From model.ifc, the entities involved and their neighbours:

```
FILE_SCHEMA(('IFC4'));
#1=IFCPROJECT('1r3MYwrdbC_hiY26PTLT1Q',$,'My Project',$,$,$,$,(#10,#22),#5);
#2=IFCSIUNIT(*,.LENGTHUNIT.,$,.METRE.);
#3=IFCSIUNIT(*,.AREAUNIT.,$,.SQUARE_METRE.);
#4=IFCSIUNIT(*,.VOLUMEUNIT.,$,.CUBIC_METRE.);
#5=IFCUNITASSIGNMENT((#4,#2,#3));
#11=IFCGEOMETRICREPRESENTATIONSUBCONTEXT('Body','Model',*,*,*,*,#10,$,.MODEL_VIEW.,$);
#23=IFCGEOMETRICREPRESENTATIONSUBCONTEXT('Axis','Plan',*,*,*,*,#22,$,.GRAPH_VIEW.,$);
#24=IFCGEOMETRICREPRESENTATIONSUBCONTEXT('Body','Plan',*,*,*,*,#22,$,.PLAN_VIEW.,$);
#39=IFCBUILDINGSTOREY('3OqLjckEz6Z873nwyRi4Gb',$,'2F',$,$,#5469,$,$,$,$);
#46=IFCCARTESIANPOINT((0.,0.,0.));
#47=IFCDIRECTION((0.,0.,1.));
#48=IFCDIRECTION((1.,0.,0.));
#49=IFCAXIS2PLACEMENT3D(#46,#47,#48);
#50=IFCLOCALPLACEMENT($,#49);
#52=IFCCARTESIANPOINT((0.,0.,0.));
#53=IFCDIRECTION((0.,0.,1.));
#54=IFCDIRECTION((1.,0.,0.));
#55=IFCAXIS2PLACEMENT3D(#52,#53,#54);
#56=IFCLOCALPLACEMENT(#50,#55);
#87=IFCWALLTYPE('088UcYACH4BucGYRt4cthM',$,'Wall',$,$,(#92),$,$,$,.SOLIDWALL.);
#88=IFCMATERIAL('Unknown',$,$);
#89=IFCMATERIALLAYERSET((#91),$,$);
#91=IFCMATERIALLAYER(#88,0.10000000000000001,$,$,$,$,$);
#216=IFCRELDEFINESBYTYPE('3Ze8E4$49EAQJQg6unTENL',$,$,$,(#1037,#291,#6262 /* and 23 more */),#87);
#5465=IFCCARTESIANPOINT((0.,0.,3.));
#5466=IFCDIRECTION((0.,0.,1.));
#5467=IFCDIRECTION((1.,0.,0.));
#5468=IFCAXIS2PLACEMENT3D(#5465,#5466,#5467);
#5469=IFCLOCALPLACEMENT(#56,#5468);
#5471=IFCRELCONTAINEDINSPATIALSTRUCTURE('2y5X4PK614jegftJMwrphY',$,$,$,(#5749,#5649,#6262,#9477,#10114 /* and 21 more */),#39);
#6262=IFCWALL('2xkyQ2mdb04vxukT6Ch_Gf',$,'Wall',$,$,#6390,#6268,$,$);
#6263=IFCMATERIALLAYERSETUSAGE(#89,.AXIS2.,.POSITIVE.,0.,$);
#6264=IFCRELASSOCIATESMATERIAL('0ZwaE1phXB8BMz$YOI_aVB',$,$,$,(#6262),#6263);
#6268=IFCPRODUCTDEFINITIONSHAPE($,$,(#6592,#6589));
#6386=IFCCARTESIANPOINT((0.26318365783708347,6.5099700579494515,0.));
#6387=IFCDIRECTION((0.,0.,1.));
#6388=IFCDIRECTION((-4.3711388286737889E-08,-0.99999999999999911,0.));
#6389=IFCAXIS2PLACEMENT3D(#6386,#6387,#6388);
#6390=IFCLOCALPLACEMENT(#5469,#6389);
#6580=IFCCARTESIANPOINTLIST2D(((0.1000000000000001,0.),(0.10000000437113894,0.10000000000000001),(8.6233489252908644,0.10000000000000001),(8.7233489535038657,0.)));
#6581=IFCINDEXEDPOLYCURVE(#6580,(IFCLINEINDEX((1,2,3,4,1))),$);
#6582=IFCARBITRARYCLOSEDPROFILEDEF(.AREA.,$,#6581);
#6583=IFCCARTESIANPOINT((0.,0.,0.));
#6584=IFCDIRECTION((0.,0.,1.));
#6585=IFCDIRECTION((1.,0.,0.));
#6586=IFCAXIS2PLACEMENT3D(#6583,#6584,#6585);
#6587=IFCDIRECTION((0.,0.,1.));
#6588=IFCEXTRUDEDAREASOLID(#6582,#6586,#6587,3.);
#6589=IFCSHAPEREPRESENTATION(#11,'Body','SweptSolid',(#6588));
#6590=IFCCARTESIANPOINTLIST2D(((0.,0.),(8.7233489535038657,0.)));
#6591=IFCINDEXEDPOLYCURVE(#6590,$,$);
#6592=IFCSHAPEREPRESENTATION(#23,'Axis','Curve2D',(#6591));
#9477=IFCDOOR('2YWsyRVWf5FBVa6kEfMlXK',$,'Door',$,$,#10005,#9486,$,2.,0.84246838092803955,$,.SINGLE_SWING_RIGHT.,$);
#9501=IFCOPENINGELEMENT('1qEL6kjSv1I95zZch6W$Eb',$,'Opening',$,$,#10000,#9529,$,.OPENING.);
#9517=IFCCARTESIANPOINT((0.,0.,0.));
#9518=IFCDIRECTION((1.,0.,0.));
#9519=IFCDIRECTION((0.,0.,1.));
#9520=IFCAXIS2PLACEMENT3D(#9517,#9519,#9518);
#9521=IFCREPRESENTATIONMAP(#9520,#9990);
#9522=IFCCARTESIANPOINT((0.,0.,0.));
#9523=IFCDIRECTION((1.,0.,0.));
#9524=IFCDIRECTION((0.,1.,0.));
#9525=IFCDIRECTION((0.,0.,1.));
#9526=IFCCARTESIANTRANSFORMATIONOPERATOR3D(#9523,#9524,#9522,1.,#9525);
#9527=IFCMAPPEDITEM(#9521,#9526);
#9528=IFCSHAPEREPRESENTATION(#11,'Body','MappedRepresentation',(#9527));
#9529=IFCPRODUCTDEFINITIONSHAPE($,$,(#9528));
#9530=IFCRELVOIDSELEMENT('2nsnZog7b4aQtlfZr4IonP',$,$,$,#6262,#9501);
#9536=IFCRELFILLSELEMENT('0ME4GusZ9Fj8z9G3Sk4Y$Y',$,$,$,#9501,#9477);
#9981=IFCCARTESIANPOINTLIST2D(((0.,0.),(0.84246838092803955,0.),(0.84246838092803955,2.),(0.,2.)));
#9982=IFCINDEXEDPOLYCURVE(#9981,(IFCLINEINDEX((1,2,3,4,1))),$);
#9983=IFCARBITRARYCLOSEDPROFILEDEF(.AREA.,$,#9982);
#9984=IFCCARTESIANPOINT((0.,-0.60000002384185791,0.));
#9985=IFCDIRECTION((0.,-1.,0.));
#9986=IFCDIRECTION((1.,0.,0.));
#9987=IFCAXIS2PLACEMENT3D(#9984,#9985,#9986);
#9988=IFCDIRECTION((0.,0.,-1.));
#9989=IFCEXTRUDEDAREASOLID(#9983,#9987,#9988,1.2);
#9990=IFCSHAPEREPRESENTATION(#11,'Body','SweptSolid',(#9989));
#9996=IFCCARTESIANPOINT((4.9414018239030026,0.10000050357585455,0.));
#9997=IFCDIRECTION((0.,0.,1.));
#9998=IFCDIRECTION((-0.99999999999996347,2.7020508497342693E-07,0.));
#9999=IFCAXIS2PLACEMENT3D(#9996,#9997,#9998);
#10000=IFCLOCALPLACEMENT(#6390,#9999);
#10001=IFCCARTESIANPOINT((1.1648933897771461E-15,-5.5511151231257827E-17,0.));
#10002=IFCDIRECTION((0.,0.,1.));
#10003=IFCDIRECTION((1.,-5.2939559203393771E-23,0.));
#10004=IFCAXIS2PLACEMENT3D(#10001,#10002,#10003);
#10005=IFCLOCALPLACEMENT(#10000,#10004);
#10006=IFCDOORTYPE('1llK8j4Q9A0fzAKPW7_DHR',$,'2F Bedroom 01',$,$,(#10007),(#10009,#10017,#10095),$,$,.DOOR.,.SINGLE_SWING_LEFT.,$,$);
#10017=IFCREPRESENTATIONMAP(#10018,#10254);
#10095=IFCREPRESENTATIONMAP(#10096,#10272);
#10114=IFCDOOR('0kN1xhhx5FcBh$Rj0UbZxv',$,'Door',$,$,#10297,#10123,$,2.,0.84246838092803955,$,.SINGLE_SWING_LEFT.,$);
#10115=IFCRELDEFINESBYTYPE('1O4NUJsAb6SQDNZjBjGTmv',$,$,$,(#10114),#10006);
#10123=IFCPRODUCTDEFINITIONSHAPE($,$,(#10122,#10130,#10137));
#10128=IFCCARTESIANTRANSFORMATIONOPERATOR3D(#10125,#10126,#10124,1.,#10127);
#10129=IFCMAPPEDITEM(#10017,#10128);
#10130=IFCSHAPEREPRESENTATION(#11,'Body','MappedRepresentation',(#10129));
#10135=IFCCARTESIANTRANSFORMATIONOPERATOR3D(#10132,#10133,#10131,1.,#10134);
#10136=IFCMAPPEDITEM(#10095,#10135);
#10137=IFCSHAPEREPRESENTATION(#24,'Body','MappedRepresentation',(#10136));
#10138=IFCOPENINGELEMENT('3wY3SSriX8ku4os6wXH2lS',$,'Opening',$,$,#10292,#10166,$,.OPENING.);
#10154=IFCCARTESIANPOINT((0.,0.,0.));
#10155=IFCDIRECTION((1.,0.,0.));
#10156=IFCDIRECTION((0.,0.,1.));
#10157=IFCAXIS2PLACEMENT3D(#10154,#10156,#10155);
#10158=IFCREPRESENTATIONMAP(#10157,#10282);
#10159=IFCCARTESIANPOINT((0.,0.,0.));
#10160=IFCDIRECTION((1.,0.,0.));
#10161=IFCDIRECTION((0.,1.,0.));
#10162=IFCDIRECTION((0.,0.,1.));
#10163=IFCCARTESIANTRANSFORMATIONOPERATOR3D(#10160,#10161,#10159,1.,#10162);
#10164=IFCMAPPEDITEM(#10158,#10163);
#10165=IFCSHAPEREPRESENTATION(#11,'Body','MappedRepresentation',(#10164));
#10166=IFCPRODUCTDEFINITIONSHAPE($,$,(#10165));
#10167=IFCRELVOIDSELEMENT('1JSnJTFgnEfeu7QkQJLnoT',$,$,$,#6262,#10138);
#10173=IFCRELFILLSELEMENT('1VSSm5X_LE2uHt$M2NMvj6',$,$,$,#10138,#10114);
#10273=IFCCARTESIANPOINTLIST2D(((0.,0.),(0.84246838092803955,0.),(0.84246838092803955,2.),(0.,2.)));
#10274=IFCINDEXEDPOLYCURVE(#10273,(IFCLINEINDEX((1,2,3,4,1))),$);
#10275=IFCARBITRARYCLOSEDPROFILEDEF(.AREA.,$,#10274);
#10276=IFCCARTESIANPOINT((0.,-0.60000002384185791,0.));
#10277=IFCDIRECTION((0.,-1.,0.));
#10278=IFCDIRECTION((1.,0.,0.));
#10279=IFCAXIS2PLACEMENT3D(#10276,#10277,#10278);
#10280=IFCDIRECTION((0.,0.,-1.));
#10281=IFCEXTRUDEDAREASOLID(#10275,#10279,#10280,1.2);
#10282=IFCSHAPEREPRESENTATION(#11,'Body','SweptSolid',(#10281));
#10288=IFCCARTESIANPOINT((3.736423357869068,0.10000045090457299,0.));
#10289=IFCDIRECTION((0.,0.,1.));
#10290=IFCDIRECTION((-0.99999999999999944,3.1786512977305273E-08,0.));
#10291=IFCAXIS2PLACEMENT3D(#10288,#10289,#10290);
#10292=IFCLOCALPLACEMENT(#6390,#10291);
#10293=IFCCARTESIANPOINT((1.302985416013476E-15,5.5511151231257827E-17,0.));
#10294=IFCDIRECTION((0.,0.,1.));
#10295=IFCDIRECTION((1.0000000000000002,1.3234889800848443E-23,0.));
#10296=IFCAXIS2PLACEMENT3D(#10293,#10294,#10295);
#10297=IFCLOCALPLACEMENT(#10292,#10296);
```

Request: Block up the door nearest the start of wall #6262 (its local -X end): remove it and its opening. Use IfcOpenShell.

```python
import ifcopenshell
import ifcopenshell.api.feature
import ifcopenshell.api.root
import ifcopenshell.geom
import ifcopenshell.util.shape

model = ifcopenshell.open("model.ifc")
settings = ifcopenshell.geom.settings()


def volume(element):
    """Net volume in cubic metres, openings subtracted."""
    shape = ifcopenshell.geom.create_shape(settings, element)
    return ifcopenshell.util.shape.get_volume(shape.geometry)


door = model.by_id(10114)
opening = door.FillsVoids[0].RelatingOpeningElement
wall = opening.VoidsElements[0].RelatingBuildingElement
before = volume(wall)

ifcopenshell.api.root.remove_product(model, product=door)
ifcopenshell.api.feature.remove_feature(model, feature=opening)

after = volume(wall)

print(f"wall volume {before:.3f} -> {after:.3f} m3")

model.write("model_updated.ifc")
```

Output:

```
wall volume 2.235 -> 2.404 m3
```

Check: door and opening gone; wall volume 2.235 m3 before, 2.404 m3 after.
